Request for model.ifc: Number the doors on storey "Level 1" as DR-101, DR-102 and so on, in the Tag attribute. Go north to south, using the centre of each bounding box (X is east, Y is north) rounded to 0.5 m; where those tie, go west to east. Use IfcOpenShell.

First a look at what the model holds.

```python
import ifcopenshell
import ifcopenshell.util.element
import ifcopenshell.util.placement

model = ifcopenshell.open("model.ifc")
print(model.schema)
storey = next(s for s in model.by_type("IfcBuildingStorey") if s.Name == "Level 1")
doors = [e for e in ifcopenshell.util.element.get_decomposition(storey) if e.is_a("IfcDoor")]
for e in sorted(doors, key=lambda e: e.id()):
    origin = ifcopenshell.util.placement.get_local_placement(e.ObjectPlacement)[:3, 3]
    print(e.id(), e.Tag, e.Name, origin.round(2) + 0.0, sep=" | ")
```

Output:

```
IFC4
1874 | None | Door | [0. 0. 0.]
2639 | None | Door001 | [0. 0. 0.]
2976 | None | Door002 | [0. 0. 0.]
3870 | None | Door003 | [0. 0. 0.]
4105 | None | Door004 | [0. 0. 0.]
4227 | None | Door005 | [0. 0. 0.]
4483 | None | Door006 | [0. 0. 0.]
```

```python
import ifcopenshell
import ifcopenshell.geom
import ifcopenshell.util.element
import ifcopenshell.util.shape

model = ifcopenshell.open("model.ifc")
settings = ifcopenshell.geom.settings()
settings.set("use-world-coords", True)


def centre(element):
    shape = ifcopenshell.geom.create_shape(settings, element)
    return ifcopenshell.util.shape.get_bbox_centroid(shape.geometry)


storey = next(s for s in model.by_type("IfcBuildingStorey") if s.Name == "Level 1")
doors = [e for e in ifcopenshell.util.element.get_decomposition(storey) if e.is_a("IfcDoor")]

# Insertion points can sit at a corner or the storey origin, so sort by the geometry (in metres).
centres = {e: centre(e) for e in doors}
doors.sort(key=lambda e: (-round(centres[e][1] / 0.5), centres[e][0]))

for i, e in enumerate(doors, start=1):
    number = f"DR-1{i:02d}"
    e.Tag = number
    print(e.id(), number)

model.write("model_v2.ifc")
```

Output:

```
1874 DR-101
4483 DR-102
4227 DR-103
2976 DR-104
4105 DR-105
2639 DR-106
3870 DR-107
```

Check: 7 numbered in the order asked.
